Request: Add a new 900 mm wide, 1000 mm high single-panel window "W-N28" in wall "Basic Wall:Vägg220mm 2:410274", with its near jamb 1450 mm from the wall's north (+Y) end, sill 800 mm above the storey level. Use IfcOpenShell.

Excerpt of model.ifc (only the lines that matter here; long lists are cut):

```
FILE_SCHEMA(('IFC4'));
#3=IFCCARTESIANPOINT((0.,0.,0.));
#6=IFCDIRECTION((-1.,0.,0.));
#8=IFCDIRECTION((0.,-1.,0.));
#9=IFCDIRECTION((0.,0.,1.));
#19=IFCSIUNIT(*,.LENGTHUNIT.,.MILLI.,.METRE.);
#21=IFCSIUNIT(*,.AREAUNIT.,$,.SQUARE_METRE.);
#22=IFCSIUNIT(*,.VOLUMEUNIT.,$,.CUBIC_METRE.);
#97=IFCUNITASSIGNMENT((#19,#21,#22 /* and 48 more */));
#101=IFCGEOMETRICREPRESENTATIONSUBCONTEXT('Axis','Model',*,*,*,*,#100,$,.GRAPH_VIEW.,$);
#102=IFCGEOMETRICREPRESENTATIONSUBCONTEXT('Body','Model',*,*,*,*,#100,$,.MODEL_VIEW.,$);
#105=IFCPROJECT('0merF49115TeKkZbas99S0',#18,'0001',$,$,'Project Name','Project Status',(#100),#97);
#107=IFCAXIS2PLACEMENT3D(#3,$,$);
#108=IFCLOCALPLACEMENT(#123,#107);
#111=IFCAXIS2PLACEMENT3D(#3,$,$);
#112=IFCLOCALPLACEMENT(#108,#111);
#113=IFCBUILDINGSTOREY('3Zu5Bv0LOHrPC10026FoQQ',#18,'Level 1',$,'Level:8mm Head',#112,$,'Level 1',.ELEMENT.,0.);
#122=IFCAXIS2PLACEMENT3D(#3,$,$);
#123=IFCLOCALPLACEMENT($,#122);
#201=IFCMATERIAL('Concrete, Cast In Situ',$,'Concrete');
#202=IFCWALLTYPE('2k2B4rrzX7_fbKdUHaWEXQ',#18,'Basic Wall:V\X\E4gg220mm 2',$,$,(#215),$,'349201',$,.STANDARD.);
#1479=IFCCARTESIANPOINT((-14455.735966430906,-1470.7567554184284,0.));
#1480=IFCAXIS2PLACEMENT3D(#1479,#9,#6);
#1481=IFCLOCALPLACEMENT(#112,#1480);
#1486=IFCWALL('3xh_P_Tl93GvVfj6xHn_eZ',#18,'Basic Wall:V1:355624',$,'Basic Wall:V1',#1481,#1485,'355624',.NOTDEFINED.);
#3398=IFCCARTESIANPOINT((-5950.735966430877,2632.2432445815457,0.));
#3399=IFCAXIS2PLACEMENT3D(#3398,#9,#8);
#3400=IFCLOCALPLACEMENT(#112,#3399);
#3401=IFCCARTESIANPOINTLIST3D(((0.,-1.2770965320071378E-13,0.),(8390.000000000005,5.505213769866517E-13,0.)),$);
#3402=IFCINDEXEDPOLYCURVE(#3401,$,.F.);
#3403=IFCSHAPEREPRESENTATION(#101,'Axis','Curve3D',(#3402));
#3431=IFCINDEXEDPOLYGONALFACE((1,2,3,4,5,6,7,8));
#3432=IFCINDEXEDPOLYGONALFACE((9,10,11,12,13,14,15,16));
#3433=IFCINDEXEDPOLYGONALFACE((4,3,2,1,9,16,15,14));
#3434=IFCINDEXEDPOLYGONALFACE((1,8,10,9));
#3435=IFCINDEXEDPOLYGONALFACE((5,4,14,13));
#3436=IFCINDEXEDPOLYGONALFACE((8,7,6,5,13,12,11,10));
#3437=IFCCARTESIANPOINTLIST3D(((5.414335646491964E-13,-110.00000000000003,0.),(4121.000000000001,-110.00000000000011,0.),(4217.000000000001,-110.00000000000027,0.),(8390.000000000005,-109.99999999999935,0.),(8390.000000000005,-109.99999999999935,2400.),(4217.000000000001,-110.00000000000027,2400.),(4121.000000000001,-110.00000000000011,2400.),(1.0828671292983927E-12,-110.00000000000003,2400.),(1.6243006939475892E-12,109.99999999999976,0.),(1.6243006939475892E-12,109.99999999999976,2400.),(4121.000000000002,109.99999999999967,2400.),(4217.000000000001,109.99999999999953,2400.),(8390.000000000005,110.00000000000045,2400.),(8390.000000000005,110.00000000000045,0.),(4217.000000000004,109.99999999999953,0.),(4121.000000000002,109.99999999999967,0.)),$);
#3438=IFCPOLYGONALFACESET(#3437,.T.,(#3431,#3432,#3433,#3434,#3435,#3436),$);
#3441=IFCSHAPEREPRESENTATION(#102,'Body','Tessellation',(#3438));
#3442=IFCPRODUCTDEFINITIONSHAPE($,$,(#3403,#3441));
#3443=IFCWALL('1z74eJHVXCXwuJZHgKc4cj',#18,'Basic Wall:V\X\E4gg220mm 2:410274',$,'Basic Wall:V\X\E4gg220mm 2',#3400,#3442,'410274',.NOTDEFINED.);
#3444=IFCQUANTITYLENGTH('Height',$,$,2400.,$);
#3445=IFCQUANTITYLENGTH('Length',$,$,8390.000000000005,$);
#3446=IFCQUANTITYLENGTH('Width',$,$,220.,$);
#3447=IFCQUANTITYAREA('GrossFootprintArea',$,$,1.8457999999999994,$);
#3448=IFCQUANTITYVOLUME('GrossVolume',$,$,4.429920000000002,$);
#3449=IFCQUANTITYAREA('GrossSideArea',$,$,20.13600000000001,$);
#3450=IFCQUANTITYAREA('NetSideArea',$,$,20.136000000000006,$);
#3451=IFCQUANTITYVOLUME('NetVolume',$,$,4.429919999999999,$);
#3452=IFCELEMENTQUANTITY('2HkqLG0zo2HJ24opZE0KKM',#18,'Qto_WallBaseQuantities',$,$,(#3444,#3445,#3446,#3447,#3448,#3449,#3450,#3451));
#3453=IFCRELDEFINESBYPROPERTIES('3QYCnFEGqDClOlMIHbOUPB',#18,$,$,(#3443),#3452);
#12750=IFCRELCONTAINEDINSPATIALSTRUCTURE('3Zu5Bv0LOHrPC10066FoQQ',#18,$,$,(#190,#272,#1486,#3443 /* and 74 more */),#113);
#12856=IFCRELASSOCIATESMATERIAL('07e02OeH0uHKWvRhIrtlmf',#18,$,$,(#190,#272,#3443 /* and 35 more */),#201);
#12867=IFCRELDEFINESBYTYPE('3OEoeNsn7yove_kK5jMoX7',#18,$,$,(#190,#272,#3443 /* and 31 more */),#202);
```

```python
import numpy as np
import ifcopenshell
import ifcopenshell.api.feature
import ifcopenshell.api.geometry
import ifcopenshell.api.pset
import ifcopenshell.api.root
import ifcopenshell.api.spatial
import ifcopenshell.geom
import ifcopenshell.util.element
import ifcopenshell.util.placement
import ifcopenshell.util.representation
import ifcopenshell.util.shape
import ifcopenshell.util.unit

model = ifcopenshell.open("model.ifc")
unit_scale = ifcopenshell.util.unit.calculate_unit_scale(model)
area_scale = ifcopenshell.util.unit.calculate_unit_scale(model, "AREAUNIT")
volume_scale = ifcopenshell.util.unit.calculate_unit_scale(model, "VOLUMEUNIT")
settings = ifcopenshell.geom.settings()


def volume(element):
    """Net volume in cubic metres, openings subtracted."""
    shape = ifcopenshell.geom.create_shape(settings, element)
    return ifcopenshell.util.shape.get_volume(shape.geometry)


wall = model.by_guid("1z74eJHVXCXwuJZHgKc4cj")
storey = ifcopenshell.util.element.get_container(wall, ifc_class="IfcBuildingStorey")
context = ifcopenshell.util.representation.get_context(model, "Model", "Body", "MODEL_VIEW")
before = volume(wall)

width, height, from_end, sill = 0.9, 1, 1.45, 0.8  # metres

# The wall runs along its own X axis, and the end named is its -X end.
wall_shape = ifcopenshell.geom.create_shape(settings, wall)
x, y, z = ifcopenshell.util.shape.get_vertices(wall_shape.geometry).T
start = x.min() + from_end
face, thickness = float(y.min()), float(y.max() - y.min())
wall_matrix = ifcopenshell.util.placement.get_local_placement(wall.ObjectPlacement)
level = ifcopenshell.util.placement.get_local_placement(storey.ObjectPlacement)[2, 3]


def in_wall(x, y):
    """Placement at x, y metres in the wall's axes, at sill height."""
    matrix = wall_matrix.copy()
    matrix[:, 3] = wall_matrix @ np.array([x / unit_scale, y / unit_scale, 0.0, 1.0])
    matrix[2, 3] = level + sill / unit_scale
    return matrix


# Opening: a box that overshoots both wall faces by 50 mm.
opening = ifcopenshell.api.root.create_entity(model, ifc_class="IfcOpeningElement", predefined_type="OPENING")
box = ifcopenshell.api.geometry.add_wall_representation(
    model, context=context, length=width, height=height, thickness=thickness + 0.1
)
ifcopenshell.api.geometry.assign_representation(model, product=opening, representation=box)
ifcopenshell.api.geometry.edit_object_placement(model, product=opening, matrix=in_wall(start, face - 0.05), is_si=False)
ifcopenshell.api.feature.add_feature(model, feature=opening, element=wall)

window = ifcopenshell.api.root.create_entity(model, ifc_class="IfcWindow", name="W-N28", predefined_type="WINDOW")
window.OverallWidth, window.OverallHeight = width / unit_scale, height / unit_scale
window.PartitioningType = "SINGLE_PANEL"
body = ifcopenshell.api.geometry.add_window_representation(
    model,
    context=context,
    overall_width=window.OverallWidth,
    overall_height=window.OverallHeight,
    partition_type="SINGLE_PANEL",
)
ifcopenshell.api.geometry.assign_representation(model, product=window, representation=body)
ifcopenshell.api.spatial.assign_container(model, products=[window], relating_structure=storey)
ifcopenshell.api.feature.add_filling(model, opening=opening, element=window)

# Centre the window in the wall's thickness.
ifcopenshell.api.geometry.edit_object_placement(model, product=window, matrix=in_wall(start, face), is_si=False)
window_shape = ifcopenshell.geom.create_shape(settings, window)
depth = ifcopenshell.util.shape.get_vertices(window_shape.geometry)[:, 1]
offset = face + thickness / 2 - (depth.min() + depth.max()) / 2
ifcopenshell.api.geometry.edit_object_placement(model, product=window, matrix=in_wall(start, offset), is_si=False)

after = volume(wall)

# Update the wall's stored quantities.
qto = model.by_id(ifcopenshell.util.element.get_pset(wall, "Qto_WallBaseQuantities", should_inherit=False)["id"])
ifcopenshell.api.pset.edit_qto(model, qto=qto, properties={
    "NetSideArea": after / thickness / area_scale,
    "NetVolume": after / volume_scale,
})

print(f"wall volume {before:.3f} -> {after:.3f} m3")

model.write("model_v2.ifc")
```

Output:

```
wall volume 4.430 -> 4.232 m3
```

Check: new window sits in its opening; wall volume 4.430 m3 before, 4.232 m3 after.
